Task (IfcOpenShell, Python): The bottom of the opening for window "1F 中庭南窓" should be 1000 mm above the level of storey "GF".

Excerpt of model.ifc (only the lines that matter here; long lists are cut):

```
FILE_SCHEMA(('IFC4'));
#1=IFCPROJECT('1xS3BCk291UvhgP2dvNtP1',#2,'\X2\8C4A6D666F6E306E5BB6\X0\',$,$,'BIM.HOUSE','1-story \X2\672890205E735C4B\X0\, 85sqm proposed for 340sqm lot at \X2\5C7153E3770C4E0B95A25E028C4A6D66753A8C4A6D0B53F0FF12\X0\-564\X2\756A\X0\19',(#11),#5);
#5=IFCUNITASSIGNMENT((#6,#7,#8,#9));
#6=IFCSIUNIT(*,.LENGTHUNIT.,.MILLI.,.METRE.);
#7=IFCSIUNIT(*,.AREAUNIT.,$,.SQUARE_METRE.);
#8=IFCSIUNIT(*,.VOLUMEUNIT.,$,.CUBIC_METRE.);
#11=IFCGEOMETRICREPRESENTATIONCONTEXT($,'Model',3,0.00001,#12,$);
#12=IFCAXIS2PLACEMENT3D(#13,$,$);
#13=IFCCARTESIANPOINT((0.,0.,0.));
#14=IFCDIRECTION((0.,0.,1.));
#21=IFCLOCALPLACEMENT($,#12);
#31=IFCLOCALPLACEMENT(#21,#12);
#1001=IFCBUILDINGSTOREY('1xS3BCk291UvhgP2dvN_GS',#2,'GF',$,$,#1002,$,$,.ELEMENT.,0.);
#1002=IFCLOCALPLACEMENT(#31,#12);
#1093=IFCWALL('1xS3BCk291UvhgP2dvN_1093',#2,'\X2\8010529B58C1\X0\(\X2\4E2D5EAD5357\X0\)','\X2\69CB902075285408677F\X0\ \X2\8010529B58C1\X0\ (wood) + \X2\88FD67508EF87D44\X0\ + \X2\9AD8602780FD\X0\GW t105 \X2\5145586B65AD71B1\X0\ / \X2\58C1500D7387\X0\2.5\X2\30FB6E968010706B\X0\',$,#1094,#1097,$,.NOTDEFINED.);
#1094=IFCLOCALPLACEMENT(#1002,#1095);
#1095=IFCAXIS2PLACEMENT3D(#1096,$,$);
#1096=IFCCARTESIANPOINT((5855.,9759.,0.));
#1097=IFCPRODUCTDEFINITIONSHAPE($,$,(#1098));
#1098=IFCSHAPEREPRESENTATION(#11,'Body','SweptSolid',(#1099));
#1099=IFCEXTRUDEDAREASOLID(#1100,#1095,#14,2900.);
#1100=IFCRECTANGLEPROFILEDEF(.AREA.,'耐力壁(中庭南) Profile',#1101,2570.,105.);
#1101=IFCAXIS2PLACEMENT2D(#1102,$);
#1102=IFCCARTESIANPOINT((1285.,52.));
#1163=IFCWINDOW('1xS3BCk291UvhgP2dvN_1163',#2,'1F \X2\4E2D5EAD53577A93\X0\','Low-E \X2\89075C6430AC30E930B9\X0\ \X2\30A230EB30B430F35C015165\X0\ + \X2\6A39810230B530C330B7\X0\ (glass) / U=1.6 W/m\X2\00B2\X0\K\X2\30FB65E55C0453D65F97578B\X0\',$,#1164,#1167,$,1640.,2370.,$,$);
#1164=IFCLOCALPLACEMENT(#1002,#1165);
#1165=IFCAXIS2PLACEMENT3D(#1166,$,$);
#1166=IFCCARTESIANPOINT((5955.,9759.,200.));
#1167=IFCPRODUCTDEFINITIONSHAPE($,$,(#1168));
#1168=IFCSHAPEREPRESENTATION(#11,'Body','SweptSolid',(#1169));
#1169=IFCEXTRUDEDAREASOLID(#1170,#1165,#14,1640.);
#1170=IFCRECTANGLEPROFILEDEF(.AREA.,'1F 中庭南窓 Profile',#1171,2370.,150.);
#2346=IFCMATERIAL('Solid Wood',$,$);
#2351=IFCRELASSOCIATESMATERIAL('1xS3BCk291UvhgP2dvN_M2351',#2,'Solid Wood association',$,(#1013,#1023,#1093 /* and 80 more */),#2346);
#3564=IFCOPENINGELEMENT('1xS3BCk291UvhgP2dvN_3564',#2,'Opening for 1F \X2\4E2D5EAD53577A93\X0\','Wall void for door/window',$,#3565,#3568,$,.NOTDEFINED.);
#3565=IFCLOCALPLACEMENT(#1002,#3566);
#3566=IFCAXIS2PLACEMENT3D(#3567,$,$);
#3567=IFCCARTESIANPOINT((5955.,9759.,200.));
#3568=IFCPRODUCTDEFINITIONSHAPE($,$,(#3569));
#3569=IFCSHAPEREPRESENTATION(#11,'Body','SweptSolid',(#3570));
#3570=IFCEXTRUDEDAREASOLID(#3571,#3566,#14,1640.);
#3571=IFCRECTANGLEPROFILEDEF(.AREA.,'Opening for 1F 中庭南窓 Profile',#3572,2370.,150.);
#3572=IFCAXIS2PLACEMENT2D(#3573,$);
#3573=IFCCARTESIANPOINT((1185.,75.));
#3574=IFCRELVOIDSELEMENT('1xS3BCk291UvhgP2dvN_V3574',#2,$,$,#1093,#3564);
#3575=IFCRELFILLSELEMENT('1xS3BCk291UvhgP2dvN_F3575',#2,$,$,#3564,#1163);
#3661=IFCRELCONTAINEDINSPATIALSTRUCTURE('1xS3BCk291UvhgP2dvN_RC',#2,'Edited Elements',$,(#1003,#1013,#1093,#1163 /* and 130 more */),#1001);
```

```python
import numpy as np
import ifcopenshell
import ifcopenshell.api.geometry
import ifcopenshell.geom
import ifcopenshell.util.element
import ifcopenshell.util.placement
import ifcopenshell.util.shape
import ifcopenshell.util.unit

model = ifcopenshell.open("model.ifc")
unit_scale = ifcopenshell.util.unit.calculate_unit_scale(model)

window = model.by_guid("1xS3BCk291UvhgP2dvN_1163")
opening = window.FillsVoids[0].RelatingOpeningElement
storey = ifcopenshell.util.element.get_container(window, ifc_class="IfcBuildingStorey")
level = ifcopenshell.util.placement.get_local_placement(storey.ObjectPlacement)[2, 3]

# The opening's origin need not be at the sill, so measure its lowest point.
shape = ifcopenshell.geom.create_shape(ifcopenshell.geom.settings(), opening)
bottom = ifcopenshell.util.shape.get_shape_bottom_elevation(shape, shape.geometry) / unit_scale
dz = level + 1 / unit_scale - bottom

shift = np.array([0.0, 0.0, dz])
# The window is not placed relative to its opening, so move both.
for product in (opening, window):
    matrix = ifcopenshell.util.placement.get_local_placement(product.ObjectPlacement)
    matrix[:3, 3] += shift
    ifcopenshell.api.geometry.edit_object_placement(model, product=product, matrix=matrix, is_si=False)

print(f"moved by {dz * unit_scale:+.3f} m")

model.write("model-out.ifc")
```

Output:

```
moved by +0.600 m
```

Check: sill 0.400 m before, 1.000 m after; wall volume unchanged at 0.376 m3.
